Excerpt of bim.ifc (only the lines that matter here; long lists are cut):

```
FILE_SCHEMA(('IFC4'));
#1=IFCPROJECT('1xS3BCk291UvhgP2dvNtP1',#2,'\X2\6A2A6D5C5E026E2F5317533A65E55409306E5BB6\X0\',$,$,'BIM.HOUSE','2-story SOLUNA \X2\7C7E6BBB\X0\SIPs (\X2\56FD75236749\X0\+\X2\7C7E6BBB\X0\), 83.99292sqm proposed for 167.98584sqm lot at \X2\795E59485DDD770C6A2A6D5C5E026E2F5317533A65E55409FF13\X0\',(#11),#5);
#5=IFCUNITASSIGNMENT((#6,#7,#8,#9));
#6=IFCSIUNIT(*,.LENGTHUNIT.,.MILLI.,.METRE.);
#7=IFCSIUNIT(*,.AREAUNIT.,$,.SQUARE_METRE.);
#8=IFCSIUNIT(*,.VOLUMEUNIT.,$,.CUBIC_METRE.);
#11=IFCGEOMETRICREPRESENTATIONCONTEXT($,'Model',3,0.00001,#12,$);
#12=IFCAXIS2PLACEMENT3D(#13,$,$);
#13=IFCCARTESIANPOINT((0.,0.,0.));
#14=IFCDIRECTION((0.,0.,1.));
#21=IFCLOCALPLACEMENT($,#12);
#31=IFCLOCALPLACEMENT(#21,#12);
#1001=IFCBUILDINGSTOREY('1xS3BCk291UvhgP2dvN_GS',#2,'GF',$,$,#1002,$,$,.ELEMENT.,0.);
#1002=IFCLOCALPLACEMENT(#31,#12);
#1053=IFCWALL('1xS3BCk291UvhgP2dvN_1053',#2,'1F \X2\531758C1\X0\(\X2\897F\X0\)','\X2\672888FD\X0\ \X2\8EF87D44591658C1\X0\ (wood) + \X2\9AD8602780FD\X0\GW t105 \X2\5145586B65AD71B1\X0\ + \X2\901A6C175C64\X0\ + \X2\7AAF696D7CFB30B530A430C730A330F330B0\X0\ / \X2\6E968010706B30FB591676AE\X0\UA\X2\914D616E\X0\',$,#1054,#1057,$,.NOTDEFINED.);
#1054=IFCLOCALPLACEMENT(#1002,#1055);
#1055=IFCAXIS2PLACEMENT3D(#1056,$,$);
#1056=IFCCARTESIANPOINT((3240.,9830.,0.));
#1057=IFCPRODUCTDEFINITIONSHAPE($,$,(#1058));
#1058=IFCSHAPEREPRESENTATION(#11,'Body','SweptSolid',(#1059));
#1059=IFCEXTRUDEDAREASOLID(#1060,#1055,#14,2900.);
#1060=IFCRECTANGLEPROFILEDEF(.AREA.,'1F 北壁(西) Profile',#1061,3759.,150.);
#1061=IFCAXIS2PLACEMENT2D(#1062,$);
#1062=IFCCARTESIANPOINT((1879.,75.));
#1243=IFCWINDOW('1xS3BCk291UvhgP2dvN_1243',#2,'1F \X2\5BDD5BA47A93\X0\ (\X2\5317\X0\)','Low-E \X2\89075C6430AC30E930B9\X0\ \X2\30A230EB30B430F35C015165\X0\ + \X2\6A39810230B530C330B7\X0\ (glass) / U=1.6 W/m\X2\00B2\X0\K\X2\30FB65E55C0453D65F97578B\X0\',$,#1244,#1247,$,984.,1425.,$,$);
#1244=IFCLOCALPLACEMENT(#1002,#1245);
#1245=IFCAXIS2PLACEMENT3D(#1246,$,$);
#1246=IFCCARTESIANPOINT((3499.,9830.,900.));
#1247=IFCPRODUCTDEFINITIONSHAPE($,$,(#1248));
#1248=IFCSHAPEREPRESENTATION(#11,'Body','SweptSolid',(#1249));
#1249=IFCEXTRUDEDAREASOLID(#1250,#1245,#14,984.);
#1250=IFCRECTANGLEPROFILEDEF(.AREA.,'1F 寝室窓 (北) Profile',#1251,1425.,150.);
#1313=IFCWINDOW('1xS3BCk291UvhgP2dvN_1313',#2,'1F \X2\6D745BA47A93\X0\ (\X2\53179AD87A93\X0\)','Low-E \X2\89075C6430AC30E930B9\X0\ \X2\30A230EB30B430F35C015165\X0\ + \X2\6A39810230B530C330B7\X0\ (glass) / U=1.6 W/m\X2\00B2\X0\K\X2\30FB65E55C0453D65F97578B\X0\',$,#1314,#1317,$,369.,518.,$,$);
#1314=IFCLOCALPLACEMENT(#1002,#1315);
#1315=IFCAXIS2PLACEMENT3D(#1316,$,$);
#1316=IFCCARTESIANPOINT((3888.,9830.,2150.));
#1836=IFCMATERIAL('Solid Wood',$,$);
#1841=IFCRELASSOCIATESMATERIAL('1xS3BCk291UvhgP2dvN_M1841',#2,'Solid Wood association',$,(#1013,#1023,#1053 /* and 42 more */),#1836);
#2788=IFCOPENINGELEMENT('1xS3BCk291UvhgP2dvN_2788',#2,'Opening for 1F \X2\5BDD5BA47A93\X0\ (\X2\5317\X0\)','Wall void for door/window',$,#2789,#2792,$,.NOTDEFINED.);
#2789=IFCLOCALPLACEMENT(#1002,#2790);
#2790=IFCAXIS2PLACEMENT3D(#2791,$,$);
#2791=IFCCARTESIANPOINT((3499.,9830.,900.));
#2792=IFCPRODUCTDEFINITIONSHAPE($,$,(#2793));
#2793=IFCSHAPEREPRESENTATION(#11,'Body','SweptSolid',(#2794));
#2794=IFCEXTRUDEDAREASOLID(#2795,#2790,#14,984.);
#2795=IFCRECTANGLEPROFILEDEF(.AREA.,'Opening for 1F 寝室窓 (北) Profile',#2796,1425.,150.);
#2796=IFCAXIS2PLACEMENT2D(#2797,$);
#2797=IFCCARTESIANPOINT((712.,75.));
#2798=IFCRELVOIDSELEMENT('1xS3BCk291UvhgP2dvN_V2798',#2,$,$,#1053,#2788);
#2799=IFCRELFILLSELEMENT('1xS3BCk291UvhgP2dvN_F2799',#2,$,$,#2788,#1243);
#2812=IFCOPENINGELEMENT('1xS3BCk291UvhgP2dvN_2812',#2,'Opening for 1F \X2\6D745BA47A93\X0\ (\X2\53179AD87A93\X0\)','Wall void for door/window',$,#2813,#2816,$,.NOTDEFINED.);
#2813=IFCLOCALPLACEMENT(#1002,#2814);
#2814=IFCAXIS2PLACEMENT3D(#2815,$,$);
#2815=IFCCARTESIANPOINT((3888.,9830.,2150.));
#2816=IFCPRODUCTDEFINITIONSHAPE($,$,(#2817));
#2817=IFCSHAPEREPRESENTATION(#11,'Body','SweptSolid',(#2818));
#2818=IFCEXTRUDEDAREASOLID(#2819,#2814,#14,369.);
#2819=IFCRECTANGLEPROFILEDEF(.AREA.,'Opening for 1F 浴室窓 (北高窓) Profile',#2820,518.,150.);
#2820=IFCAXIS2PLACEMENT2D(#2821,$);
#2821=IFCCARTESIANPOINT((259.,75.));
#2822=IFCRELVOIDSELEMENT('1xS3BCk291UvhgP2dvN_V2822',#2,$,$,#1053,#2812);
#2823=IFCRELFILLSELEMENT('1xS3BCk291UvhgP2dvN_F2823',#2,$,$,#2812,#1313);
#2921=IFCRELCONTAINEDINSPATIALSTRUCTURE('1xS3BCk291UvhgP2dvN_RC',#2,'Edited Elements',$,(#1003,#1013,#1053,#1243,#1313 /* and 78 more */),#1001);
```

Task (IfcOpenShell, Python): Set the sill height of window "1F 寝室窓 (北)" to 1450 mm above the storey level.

```python
import numpy as np
import ifcopenshell
import ifcopenshell.api.geometry
import ifcopenshell.geom
import ifcopenshell.util.element
import ifcopenshell.util.placement
import ifcopenshell.util.shape
import ifcopenshell.util.unit

model = ifcopenshell.open("bim.ifc")
unit_scale = ifcopenshell.util.unit.calculate_unit_scale(model)

window = model.by_guid("1xS3BCk291UvhgP2dvN_1243")
opening = window.FillsVoids[0].RelatingOpeningElement
storey = ifcopenshell.util.element.get_container(window, ifc_class="IfcBuildingStorey")
level = ifcopenshell.util.placement.get_local_placement(storey.ObjectPlacement)[2, 3]

# The opening's origin need not be at the sill, so measure its lowest point.
shape = ifcopenshell.geom.create_shape(ifcopenshell.geom.settings(), opening)
bottom = ifcopenshell.util.shape.get_shape_bottom_elevation(shape, shape.geometry) / unit_scale
dz = level + 1.45 / unit_scale - bottom

shift = np.array([0.0, 0.0, dz])
# The window is not placed relative to its opening, so move both.
for product in (opening, window):
    matrix = ifcopenshell.util.placement.get_local_placement(product.ObjectPlacement)
    matrix[:3, 3] += shift
    ifcopenshell.api.geometry.edit_object_placement(model, product=product, matrix=matrix, is_si=False)

print(f"moved by {dz * unit_scale:+.3f} m")

model.write("bim-out.ifc")
```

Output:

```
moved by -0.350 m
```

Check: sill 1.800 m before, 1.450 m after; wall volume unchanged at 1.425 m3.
